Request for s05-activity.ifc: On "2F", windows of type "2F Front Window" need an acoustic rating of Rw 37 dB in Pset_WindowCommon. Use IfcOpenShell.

First a look at what the model holds.

```python
import ifcopenshell
import ifcopenshell.util.element

model = ifcopenshell.open("s05-activity.ifc")
print(model.schema)
storey = next(s for s in model.by_type("IfcBuildingStorey") if s.Name == "2F")
windows = [e for e in ifcopenshell.util.element.get_decomposition(storey) if e.is_a("IfcWindow")]
seen = {}
for e in windows:
    element_type = ifcopenshell.util.element.get_type(e)
    key = (element_type.Name if element_type != e and element_type else None, ifcopenshell.util.element.get_pset(e, "Pset_WindowCommon", "AcousticRating"))
    seen[key] = seen.get(key, 0) + 1
for (name, value), count in sorted(seen.items(), key=str):
    print(count, "x", name, "|", value)
```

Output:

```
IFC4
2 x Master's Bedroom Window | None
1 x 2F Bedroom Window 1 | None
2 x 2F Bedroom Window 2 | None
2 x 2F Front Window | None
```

```python
import ifcopenshell
import ifcopenshell.api.pset
import ifcopenshell.util.element

model = ifcopenshell.open("s05-activity.ifc")

storey = next(s for s in model.by_type("IfcBuildingStorey") if s.Name == "2F")
windows = [e for e in ifcopenshell.util.element.get_decomposition(storey) if e.is_a("IfcWindow")]

count = 0
for e in windows:
    element_type = ifcopenshell.util.element.get_type(e)
    if element_type in (None, e) or element_type.Name != "2F Front Window":
        continue
    # add_pset returns the element's existing set when there is one.
    pset = ifcopenshell.api.pset.add_pset(model, product=e, name="Pset_WindowCommon")
    ifcopenshell.api.pset.edit_pset(model, pset=pset, properties={"AcousticRating": "Rw 37 dB"})
    count += 1

print(count, "windows updated")

model.write("s05-activity_updated.ifc")
```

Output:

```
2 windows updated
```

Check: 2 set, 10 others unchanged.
